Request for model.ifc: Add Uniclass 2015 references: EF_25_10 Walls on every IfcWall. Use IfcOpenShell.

First a look at what the model holds.

```python
import ifcopenshell

model = ifcopenshell.open("model.ifc")
print(model.schema)
print("classifications:", [c.Name for c in model.by_type("IfcClassification")])
for ifc_class in ("IfcDoor", "IfcRoof", "IfcStair", "IfcWall", "IfcWindow"):
    print(ifc_class, len(model.by_type(ifc_class)))
```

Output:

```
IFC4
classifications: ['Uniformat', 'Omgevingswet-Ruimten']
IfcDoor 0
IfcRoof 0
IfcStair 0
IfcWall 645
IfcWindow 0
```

```python
import ifcopenshell
import ifcopenshell.api.classification

model = ifcopenshell.open("model.ifc")

system = ifcopenshell.api.classification.add_classification(model, classification="Uniclass 2015")

codes = {
    "IfcWall": ("EF_25_10", "Walls"),
}
for ifc_class, (code, name) in codes.items():
    products = model.by_type(ifc_class)
    ifcopenshell.api.classification.add_reference(
        model, products=products, classification=system, identification=code, name=name
    )
    print(code, len(products))

model.write("model_v2.ifc")
```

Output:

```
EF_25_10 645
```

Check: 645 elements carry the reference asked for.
